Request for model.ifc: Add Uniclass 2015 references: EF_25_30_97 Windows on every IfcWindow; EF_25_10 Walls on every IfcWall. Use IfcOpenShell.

First a look at what the model holds.

```python
import ifcopenshell

model = ifcopenshell.open("model.ifc")
print(model.schema)
print("classifications:", [c.Name for c in model.by_type("IfcClassification")])
for ifc_class in ("IfcDoor", "IfcRoof", "IfcStair", "IfcWall", "IfcWindow"):
    print(ifc_class, len(model.by_type(ifc_class)))
```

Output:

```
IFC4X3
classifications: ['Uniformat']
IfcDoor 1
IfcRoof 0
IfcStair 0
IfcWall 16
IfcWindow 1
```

```python
import ifcopenshell
import ifcopenshell.api.classification

model = ifcopenshell.open("model.ifc")

system = ifcopenshell.api.classification.add_classification(model, classification="Uniclass 2015")

codes = {
    "IfcWindow": ("EF_25_30_97", "Windows"),
    "IfcWall": ("EF_25_10", "Walls"),
}
for ifc_class, (code, name) in codes.items():
    products = model.by_type(ifc_class)
    ifcopenshell.api.classification.add_reference(
        model, products=products, classification=system, identification=code, name=name
    )
    print(code, len(products))

model.write("model_v2.ifc")
```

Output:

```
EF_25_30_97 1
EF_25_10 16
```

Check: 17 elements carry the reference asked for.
